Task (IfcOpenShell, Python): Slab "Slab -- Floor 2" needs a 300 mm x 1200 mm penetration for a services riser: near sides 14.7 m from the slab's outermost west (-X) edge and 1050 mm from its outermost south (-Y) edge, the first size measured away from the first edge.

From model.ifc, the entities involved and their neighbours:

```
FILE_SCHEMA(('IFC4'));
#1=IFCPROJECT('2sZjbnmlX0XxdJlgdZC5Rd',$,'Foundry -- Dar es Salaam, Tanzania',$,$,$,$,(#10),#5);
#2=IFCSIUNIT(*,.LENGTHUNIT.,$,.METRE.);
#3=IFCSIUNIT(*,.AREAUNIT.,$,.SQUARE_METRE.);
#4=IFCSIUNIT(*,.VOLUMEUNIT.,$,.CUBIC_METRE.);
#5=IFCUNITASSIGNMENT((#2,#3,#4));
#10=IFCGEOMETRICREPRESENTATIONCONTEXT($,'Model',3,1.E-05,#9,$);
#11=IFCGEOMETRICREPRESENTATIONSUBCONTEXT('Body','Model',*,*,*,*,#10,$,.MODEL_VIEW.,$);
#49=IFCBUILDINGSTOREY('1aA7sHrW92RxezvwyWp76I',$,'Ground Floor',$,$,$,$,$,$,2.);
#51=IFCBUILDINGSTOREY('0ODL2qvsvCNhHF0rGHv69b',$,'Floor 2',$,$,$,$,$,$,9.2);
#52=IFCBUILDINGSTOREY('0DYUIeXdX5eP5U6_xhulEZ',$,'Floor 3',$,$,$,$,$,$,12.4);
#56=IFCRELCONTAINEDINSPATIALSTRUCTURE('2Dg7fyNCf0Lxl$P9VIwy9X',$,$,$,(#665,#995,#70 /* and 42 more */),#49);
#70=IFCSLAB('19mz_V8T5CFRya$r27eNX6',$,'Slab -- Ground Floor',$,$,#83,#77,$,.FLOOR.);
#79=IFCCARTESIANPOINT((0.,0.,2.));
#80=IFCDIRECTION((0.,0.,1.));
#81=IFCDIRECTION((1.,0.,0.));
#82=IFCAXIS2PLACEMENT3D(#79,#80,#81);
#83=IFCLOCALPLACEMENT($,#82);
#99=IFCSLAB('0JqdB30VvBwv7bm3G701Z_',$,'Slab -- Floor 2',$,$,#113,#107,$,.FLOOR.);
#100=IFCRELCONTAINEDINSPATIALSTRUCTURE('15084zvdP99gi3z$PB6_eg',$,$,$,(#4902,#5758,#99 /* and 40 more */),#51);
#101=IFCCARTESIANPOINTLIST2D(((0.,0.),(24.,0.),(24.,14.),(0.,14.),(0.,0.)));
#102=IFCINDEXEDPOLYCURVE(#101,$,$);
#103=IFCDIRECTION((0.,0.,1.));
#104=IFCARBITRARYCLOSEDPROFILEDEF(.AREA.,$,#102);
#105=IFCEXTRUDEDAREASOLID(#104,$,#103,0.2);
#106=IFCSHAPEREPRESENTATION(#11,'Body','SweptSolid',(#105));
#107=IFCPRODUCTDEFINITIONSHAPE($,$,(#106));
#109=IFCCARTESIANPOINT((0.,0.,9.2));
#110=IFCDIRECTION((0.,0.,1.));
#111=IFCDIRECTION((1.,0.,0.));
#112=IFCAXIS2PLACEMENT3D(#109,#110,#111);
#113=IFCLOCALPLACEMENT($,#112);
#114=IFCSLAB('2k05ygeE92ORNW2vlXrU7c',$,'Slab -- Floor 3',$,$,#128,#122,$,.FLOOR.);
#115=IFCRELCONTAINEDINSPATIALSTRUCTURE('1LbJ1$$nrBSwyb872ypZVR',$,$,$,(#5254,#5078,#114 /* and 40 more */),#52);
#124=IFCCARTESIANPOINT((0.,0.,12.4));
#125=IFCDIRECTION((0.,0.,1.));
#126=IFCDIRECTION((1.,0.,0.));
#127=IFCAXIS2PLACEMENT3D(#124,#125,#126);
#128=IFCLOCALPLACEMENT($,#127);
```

```python
import numpy as np
import ifcopenshell
import ifcopenshell.api.feature
import ifcopenshell.api.geometry
import ifcopenshell.api.root
import ifcopenshell.geom
import ifcopenshell.util.placement
import ifcopenshell.util.representation
import ifcopenshell.util.shape
import ifcopenshell.util.unit

model = ifcopenshell.open("model.ifc")
unit_scale = ifcopenshell.util.unit.calculate_unit_scale(model)
settings = ifcopenshell.geom.settings()


def volume(element):
    """Net volume in cubic metres, openings subtracted."""
    shape = ifcopenshell.geom.create_shape(settings, element)
    return ifcopenshell.util.shape.get_volume(shape.geometry)


slab = model.by_id(99)
before = volume(slab)

# Extent in the slab's own axes, in metres. The edges named are its -X and -Y sides.
slab_shape = ifcopenshell.geom.create_shape(settings, slab)
vertices = ifcopenshell.util.shape.get_vertices(slab_shape.geometry)
x_min, y_min, bottom = vertices.min(axis=0)
top = vertices[:, 2].max()

opening = ifcopenshell.api.root.create_entity(model, ifc_class="IfcOpeningElement", name="Services riser opening", predefined_type="OPENING")
context = ifcopenshell.util.representation.get_context(model, "Model", "Body", "MODEL_VIEW")
width, depth = 0.3, 1.2
outline = [(0.0, 0.0), (width, 0.0), (width, depth), (0.0, depth), (0.0, 0.0)]
# Overshoot both faces by 50 mm so the cut is clean.
shape = ifcopenshell.api.geometry.add_slab_representation(
    model, context=context, depth=top - bottom + 0.1, polyline=outline
)
ifcopenshell.api.geometry.assign_representation(model, product=opening, representation=shape)

matrix = ifcopenshell.util.placement.get_local_placement(slab.ObjectPlacement)
matrix[:, 3] = matrix @ np.append(np.array([x_min + 14.7, y_min + 1.05, bottom - 0.05]) / unit_scale, 1.0)
ifcopenshell.api.geometry.edit_object_placement(model, product=opening, matrix=matrix, is_si=False)
ifcopenshell.api.feature.add_feature(model, feature=opening, element=slab)

after = volume(slab)

print(f"slab volume {before:.3f} -> {after:.3f} m3")

model.write("model_rev.ifc")
```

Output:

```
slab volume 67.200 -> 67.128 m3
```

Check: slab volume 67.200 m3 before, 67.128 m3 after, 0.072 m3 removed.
